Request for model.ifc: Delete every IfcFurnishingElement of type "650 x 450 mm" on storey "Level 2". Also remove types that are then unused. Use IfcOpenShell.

First a look at what the model holds.

```python
import ifcopenshell
import ifcopenshell.util.element

model = ifcopenshell.open("model.ifc")
print(model.schema)
storey = next(s for s in model.by_type("IfcBuildingStorey") if s.Name == "Level 2")
furniture = [e for e in ifcopenshell.util.element.get_decomposition(storey) if e.is_a("IfcFurnishingElement")]
seen = {}
for e in furniture:
    element_type = ifcopenshell.util.element.get_type(e)
    name = element_type.Name if element_type not in (None, e) else None
    seen[name] = seen.get(name, 0) + 1
for name, count in sorted(seen.items(), key=str):
    print(count, "x", name)
```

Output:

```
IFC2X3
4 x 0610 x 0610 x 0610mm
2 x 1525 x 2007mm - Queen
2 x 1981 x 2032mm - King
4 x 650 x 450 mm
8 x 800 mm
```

```python
import ifcopenshell
import ifcopenshell.api.root
import ifcopenshell.util.element

model = ifcopenshell.open("model.ifc")

storey = next(s for s in model.by_type("IfcBuildingStorey") if s.Name == "Level 2")
furniture = [e for e in ifcopenshell.util.element.get_decomposition(storey) if e.is_a("IfcFurnishingElement")]
targets = [e for e in furniture if (t := ifcopenshell.util.element.get_type(e)) not in (None, e) and t.Name == "650 x 450 mm"]
types = {ifcopenshell.util.element.get_type(e) for e in targets} - {None, *targets}

for e in targets:
    ifcopenshell.api.root.remove_product(model, product=e)
print(len(targets), "removed")

unused = [t for t in types if not ifcopenshell.util.element.get_types(t)]
for t in unused:
    ifcopenshell.api.root.remove_product(model, product=t)
print(len(unused), "unused types removed")

model.write("model_edited.ifc")
```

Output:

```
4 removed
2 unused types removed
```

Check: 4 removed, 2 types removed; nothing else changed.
